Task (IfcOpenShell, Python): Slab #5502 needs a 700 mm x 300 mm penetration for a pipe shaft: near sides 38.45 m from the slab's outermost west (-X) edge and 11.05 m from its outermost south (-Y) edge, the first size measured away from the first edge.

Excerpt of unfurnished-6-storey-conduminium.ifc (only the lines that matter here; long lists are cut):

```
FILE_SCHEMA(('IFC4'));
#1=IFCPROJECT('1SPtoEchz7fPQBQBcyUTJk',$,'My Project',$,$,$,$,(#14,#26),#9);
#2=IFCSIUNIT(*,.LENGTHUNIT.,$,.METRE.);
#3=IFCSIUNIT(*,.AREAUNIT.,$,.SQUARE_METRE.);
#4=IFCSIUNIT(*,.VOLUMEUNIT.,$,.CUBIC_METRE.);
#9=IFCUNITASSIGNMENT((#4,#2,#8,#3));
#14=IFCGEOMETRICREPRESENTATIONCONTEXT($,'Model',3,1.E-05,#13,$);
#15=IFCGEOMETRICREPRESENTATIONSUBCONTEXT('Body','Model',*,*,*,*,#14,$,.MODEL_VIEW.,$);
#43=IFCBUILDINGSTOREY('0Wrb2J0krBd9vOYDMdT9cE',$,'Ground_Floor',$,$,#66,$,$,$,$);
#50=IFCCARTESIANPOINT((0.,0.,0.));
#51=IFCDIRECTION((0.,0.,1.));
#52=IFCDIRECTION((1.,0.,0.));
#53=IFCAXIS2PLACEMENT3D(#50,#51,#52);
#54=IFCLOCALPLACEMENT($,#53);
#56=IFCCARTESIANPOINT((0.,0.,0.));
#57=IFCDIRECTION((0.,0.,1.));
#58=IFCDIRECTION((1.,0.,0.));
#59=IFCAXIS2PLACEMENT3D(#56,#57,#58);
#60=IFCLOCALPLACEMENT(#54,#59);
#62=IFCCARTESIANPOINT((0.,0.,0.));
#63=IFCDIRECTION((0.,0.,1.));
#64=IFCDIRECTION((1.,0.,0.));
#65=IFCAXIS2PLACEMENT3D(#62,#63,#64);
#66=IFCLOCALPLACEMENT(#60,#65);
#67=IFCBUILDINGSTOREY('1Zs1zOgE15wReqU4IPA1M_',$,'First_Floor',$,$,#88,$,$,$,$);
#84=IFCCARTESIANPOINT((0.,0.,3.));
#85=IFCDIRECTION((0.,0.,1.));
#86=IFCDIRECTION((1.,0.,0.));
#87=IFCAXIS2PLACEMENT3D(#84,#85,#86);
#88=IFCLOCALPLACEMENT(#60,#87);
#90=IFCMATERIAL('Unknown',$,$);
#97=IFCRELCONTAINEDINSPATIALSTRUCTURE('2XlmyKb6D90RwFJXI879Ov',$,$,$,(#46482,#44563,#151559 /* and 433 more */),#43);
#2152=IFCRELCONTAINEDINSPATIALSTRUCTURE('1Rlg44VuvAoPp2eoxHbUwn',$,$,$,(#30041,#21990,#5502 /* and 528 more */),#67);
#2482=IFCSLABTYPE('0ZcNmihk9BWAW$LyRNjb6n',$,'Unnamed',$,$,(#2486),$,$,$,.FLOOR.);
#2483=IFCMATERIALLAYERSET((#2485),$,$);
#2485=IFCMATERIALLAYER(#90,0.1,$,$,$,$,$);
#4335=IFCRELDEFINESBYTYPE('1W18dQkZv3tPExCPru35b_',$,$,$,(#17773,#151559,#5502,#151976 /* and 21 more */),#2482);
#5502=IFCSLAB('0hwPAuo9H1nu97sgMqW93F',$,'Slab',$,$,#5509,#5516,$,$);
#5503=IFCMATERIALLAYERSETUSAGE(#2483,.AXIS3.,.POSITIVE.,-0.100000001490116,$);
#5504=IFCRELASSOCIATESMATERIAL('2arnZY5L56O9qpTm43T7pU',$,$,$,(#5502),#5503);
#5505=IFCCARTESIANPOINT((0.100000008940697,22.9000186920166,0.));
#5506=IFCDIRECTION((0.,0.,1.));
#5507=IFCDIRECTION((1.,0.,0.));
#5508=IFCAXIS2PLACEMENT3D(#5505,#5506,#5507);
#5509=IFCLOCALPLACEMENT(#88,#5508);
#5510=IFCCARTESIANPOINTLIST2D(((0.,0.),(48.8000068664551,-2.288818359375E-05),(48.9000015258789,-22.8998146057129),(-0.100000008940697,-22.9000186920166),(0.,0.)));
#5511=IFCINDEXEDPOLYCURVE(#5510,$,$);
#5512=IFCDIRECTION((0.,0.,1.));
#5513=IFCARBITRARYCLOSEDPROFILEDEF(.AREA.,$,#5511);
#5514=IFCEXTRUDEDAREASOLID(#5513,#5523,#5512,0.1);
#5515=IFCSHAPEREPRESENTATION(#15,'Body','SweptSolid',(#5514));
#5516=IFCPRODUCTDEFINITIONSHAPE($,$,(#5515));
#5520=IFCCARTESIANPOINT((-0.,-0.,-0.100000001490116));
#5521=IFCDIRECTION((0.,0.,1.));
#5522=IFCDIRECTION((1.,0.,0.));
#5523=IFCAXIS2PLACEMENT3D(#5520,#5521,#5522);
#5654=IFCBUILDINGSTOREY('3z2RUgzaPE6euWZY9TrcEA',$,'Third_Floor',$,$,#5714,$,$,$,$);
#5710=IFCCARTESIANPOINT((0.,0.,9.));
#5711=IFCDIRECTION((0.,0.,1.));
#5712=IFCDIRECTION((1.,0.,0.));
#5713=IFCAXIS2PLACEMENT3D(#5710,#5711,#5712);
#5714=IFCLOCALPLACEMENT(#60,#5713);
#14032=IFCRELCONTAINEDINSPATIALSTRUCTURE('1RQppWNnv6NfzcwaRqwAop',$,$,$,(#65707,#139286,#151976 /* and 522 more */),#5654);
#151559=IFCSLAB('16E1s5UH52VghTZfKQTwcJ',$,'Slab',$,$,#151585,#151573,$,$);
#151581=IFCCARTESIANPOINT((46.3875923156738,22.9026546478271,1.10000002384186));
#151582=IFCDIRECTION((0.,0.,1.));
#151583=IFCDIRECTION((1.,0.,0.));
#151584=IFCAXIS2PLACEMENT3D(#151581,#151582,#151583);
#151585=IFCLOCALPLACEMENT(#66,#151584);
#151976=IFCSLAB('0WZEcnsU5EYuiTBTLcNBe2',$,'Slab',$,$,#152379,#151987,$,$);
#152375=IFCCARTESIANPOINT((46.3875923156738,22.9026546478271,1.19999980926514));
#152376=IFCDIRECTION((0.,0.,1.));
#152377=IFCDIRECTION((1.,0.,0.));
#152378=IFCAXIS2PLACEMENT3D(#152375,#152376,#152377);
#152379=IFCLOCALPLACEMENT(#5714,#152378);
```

```python
import numpy as np
import ifcopenshell
import ifcopenshell.api.feature
import ifcopenshell.api.geometry
import ifcopenshell.api.root
import ifcopenshell.geom
import ifcopenshell.util.placement
import ifcopenshell.util.representation
import ifcopenshell.util.shape
import ifcopenshell.util.unit

model = ifcopenshell.open("unfurnished-6-storey-conduminium.ifc")
unit_scale = ifcopenshell.util.unit.calculate_unit_scale(model)
settings = ifcopenshell.geom.settings()


def volume(element):
    """Net volume in cubic metres, openings subtracted."""
    shape = ifcopenshell.geom.create_shape(settings, element)
    return ifcopenshell.util.shape.get_volume(shape.geometry)


slab = model.by_guid("0hwPAuo9H1nu97sgMqW93F")
before = volume(slab)

# Extent in the slab's own axes, in metres. The edges named are its -X and -Y sides.
slab_shape = ifcopenshell.geom.create_shape(settings, slab)
vertices = ifcopenshell.util.shape.get_vertices(slab_shape.geometry)
x_min, y_min, bottom = vertices.min(axis=0)
top = vertices[:, 2].max()

opening = ifcopenshell.api.root.create_entity(model, ifc_class="IfcOpeningElement", name="Pipe shaft opening", predefined_type="OPENING")
context = ifcopenshell.util.representation.get_context(model, "Model", "Body", "MODEL_VIEW")
width, depth = 0.7, 0.3
outline = [(0.0, 0.0), (width, 0.0), (width, depth), (0.0, depth), (0.0, 0.0)]
# Overshoot both faces by 50 mm so the cut is clean.
shape = ifcopenshell.api.geometry.add_slab_representation(
    model, context=context, depth=top - bottom + 0.1, polyline=outline
)
ifcopenshell.api.geometry.assign_representation(model, product=opening, representation=shape)

matrix = ifcopenshell.util.placement.get_local_placement(slab.ObjectPlacement)
matrix[:, 3] = matrix @ np.append(np.array([x_min + 38.45, y_min + 11.05, bottom - 0.05]) / unit_scale, 1.0)
ifcopenshell.api.geometry.edit_object_placement(model, product=opening, matrix=matrix, is_si=False)
ifcopenshell.api.feature.add_feature(model, feature=opening, element=slab)

after = volume(slab)

print(f"slab volume {before:.3f} -> {after:.3f} m3")

model.write("unfurnished-6-storey-conduminium_rev.ifc")
```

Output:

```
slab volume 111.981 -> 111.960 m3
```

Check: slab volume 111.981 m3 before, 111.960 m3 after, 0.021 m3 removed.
